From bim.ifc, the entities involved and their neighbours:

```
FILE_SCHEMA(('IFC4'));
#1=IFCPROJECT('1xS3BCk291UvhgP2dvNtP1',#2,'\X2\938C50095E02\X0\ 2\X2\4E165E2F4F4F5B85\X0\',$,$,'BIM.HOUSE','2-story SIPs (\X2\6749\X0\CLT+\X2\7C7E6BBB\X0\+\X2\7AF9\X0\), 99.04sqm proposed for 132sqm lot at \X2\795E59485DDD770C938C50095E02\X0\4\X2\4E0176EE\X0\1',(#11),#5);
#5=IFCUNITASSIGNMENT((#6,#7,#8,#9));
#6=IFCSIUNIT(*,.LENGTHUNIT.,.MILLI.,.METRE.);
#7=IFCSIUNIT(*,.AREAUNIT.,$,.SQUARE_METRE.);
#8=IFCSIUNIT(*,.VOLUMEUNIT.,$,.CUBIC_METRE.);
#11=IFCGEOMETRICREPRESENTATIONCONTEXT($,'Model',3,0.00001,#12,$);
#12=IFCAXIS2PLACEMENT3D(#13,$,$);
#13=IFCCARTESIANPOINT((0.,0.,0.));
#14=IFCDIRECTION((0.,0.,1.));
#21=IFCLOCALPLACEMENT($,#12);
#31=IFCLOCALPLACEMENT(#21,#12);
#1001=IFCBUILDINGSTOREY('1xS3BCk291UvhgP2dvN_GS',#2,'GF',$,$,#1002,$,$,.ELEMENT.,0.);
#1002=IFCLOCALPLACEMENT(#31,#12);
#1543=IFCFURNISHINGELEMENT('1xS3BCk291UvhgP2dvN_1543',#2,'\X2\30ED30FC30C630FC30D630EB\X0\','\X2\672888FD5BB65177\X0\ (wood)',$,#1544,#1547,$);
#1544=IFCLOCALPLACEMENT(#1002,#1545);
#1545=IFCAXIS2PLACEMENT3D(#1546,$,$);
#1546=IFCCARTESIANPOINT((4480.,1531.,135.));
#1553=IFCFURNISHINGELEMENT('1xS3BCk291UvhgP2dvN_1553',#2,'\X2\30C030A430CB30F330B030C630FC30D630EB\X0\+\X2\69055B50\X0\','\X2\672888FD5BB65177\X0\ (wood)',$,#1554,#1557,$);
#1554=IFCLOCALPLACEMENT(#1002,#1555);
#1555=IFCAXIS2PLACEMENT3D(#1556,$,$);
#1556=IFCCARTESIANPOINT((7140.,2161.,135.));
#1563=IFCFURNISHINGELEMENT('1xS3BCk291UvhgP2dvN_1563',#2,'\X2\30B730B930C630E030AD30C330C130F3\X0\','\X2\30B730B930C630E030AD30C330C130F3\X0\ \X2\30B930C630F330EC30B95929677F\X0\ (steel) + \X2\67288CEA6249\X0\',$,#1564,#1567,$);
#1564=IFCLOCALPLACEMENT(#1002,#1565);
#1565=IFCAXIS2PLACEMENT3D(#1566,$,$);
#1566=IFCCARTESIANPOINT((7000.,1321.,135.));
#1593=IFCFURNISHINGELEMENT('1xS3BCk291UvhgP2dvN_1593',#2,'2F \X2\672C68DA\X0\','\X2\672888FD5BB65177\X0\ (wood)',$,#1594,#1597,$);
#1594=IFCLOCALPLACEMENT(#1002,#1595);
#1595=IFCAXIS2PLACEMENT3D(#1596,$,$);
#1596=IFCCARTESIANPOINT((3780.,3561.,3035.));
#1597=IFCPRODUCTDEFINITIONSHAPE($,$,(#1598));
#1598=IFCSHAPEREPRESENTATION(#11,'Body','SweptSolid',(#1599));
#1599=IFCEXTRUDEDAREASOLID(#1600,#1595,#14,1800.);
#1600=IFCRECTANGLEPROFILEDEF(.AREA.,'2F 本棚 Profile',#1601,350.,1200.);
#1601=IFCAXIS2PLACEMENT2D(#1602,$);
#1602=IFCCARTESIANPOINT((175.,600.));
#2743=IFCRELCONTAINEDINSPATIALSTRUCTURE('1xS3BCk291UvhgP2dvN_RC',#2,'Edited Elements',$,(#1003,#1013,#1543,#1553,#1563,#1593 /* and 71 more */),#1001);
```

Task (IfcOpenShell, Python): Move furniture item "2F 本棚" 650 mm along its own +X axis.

```python
import ifcopenshell
import ifcopenshell.api.geometry
import ifcopenshell.util.placement
import ifcopenshell.util.unit

model = ifcopenshell.open("bim.ifc")
unit_scale = ifcopenshell.util.unit.calculate_unit_scale(model)

item = model.by_guid("1xS3BCk291UvhgP2dvN_1593")
matrix = ifcopenshell.util.placement.get_local_placement(item.ObjectPlacement)
matrix[:3, 3] += matrix[:3, 0] * 0.65 / unit_scale
ifcopenshell.api.geometry.edit_object_placement(model, product=item, matrix=matrix, is_si=False)

print(ifcopenshell.util.placement.get_local_placement(item.ObjectPlacement).round(3) + 0.0)

model.write("bim_edited.ifc")
```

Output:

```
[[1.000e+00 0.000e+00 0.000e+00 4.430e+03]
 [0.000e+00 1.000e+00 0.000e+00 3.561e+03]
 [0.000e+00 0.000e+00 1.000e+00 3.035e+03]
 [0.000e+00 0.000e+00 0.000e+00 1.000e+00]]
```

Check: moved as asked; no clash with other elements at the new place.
